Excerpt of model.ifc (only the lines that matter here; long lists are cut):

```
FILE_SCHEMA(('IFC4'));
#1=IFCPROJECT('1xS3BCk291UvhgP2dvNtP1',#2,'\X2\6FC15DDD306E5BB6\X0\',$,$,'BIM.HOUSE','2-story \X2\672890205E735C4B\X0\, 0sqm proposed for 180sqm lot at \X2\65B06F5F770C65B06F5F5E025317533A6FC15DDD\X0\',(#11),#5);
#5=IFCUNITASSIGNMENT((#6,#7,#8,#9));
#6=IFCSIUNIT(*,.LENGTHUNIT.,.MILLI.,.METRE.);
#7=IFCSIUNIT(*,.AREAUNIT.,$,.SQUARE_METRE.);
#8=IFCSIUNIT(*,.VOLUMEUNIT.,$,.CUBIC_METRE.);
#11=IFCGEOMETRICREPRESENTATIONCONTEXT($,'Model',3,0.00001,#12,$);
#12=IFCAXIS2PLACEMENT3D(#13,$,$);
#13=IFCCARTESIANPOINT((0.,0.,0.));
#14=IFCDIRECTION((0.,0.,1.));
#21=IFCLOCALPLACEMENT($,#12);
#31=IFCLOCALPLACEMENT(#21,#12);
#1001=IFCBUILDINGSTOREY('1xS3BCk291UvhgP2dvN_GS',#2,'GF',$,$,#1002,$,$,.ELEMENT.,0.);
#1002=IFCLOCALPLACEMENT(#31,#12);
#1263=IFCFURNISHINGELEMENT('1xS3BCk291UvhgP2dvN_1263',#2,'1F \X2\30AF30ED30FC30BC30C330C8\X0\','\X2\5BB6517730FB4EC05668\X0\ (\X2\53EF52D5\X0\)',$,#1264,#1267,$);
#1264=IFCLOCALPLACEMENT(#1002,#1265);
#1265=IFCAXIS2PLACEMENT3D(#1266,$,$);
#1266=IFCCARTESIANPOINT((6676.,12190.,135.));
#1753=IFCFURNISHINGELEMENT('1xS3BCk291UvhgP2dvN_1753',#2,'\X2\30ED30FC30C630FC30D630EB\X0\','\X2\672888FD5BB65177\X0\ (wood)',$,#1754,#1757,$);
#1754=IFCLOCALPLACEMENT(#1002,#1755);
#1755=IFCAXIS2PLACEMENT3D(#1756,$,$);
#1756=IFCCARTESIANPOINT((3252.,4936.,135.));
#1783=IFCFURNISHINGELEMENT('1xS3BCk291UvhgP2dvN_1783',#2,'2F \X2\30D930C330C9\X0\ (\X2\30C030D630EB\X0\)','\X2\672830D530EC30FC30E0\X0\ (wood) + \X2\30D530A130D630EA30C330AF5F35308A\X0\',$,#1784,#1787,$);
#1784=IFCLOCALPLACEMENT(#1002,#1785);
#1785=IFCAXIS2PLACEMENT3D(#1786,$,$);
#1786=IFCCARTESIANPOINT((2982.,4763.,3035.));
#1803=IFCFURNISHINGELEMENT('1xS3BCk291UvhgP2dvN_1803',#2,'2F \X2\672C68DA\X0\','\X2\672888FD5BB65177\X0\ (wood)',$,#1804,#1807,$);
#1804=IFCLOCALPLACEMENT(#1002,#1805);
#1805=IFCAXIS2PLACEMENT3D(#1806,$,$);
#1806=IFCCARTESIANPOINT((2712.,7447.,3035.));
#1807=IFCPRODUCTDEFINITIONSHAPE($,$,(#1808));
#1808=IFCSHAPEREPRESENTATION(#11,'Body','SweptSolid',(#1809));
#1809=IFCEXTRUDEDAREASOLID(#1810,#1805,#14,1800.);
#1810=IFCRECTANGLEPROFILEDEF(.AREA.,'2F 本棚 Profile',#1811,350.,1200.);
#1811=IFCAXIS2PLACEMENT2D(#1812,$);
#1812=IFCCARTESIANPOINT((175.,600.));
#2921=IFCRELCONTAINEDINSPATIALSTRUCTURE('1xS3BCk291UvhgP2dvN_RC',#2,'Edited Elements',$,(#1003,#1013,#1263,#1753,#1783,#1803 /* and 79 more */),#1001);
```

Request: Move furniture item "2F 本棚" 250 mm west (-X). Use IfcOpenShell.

```python
import ifcopenshell
import ifcopenshell.api.geometry
import ifcopenshell.util.placement

model = ifcopenshell.open("model.ifc")

item = model.by_guid("1xS3BCk291UvhgP2dvN_1803")
matrix = ifcopenshell.util.placement.get_local_placement(item.ObjectPlacement)
matrix[0, 3] -= 250.0
ifcopenshell.api.geometry.edit_object_placement(model, product=item, matrix=matrix, is_si=False)

print(ifcopenshell.util.placement.get_local_placement(item.ObjectPlacement).round(3) + 0.0)

model.write("model_rev.ifc")
```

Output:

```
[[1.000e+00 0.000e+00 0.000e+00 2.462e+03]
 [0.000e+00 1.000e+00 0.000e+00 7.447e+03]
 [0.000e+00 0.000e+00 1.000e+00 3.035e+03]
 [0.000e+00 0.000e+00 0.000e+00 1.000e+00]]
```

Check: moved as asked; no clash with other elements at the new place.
